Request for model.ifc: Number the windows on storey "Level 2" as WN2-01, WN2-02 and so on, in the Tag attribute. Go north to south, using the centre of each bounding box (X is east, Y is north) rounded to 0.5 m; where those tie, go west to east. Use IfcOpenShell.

First a look at what the model holds.

```python
import ifcopenshell
import ifcopenshell.util.element
import ifcopenshell.util.placement

model = ifcopenshell.open("model.ifc")
print(model.schema)
storey = next(s for s in model.by_type("IfcBuildingStorey") if s.Name == "Level 2")
windows = [e for e in ifcopenshell.util.element.get_decomposition(storey) if e.is_a("IfcWindow")]
for e in sorted(windows, key=lambda e: e.id()):
    origin = ifcopenshell.util.placement.get_local_placement(e.ObjectPlacement)[:3, 3]
    print(e.id(), e.Tag, e.Name, origin.round(2) + 0.0, sep=" | ")
```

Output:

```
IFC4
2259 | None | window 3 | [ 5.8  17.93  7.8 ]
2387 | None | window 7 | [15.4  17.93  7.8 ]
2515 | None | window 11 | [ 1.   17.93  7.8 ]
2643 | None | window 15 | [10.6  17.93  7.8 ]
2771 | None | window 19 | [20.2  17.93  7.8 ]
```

```python
import ifcopenshell
import ifcopenshell.geom
import ifcopenshell.util.element
import ifcopenshell.util.shape

model = ifcopenshell.open("model.ifc")
settings = ifcopenshell.geom.settings()
settings.set("use-world-coords", True)


def centre(element):
    shape = ifcopenshell.geom.create_shape(settings, element)
    return ifcopenshell.util.shape.get_bbox_centroid(shape.geometry)


storey = next(s for s in model.by_type("IfcBuildingStorey") if s.Name == "Level 2")
windows = [e for e in ifcopenshell.util.element.get_decomposition(storey) if e.is_a("IfcWindow")]

# Insertion points can sit at a corner or the storey origin, so sort by the geometry (in metres).
centres = {e: centre(e) for e in windows}
windows.sort(key=lambda e: (-round(centres[e][1] / 0.5), centres[e][0]))

for i, e in enumerate(windows, start=1):
    number = f"WN2-{i:02d}"
    e.Tag = number
    print(e.id(), number)

model.write("model_v2.ifc")
```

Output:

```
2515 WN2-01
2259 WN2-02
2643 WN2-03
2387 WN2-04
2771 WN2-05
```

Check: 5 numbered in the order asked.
